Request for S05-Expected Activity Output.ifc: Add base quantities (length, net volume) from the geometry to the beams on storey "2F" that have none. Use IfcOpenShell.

First a look at what the model holds.

```python
import ifcopenshell
import ifcopenshell.util.element
import ifcopenshell.util.unit

model = ifcopenshell.open("S05-Expected Activity Output.ifc")
print(model.schema)
for unit_type in ("LENGTHUNIT", "AREAUNIT", "VOLUMEUNIT"):
    print(unit_type, ifcopenshell.util.unit.calculate_unit_scale(model, unit_type))
storey = next(s for s in model.by_type("IfcBuildingStorey") if s.Name == "2F")
beams = [e for e in ifcopenshell.util.element.get_decomposition(storey) if e.is_a("IfcBeam")]
for e in sorted(beams, key=lambda e: e.id()):
    print(e.id(), e.is_a(), e.Name, list(ifcopenshell.util.element.get_psets(e, qtos_only=True)), sep=" | ")
```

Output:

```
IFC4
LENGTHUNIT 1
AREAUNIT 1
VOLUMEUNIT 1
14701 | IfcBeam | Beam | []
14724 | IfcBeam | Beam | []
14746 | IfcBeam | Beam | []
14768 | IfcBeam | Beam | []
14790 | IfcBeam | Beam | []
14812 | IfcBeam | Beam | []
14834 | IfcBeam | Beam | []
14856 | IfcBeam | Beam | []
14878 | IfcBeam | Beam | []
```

```python
import ifcopenshell
import ifcopenshell.api.pset
import ifcopenshell.geom
import ifcopenshell.util.element
import ifcopenshell.util.shape
import ifcopenshell.util.unit

model = ifcopenshell.open("S05-Expected Activity Output.ifc")
unit_scale = ifcopenshell.util.unit.calculate_unit_scale(model)
volume_scale = ifcopenshell.util.unit.calculate_unit_scale(model, "VOLUMEUNIT")
settings = ifcopenshell.geom.settings()

storey = next(s for s in model.by_type("IfcBuildingStorey") if s.Name == "2F")
beams = [e for e in ifcopenshell.util.element.get_decomposition(storey) if e.is_a("IfcBeam")]

for e in sorted(beams, key=lambda e: e.id()):
    if ifcopenshell.util.element.get_psets(e, qtos_only=True, should_inherit=False):
        continue
    # Geometry comes back in metres, in the element's own axes.
    shape = ifcopenshell.geom.create_shape(settings, e)
    values = {
        "Length": ifcopenshell.util.shape.get_max_xyz(shape.geometry) / unit_scale,
        "NetVolume": ifcopenshell.util.shape.get_volume(shape.geometry) / volume_scale,
    }
    qto = ifcopenshell.api.pset.add_qto(model, product=e, name="Qto_BeamBaseQuantities")
    ifcopenshell.api.pset.edit_qto(model, qto=qto, properties=values)
    print(e.id(), {k: round(v, 3) for k, v in values.items()})

model.write("S05-Expected Activity Output_v2.ifc")
```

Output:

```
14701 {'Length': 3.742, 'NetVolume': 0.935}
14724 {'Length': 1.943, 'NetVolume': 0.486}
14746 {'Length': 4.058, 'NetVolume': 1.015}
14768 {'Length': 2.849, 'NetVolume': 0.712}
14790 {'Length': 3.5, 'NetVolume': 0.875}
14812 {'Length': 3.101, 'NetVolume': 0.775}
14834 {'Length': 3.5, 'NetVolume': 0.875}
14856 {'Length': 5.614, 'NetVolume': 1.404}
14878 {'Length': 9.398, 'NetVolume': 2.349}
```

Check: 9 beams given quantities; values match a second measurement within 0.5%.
